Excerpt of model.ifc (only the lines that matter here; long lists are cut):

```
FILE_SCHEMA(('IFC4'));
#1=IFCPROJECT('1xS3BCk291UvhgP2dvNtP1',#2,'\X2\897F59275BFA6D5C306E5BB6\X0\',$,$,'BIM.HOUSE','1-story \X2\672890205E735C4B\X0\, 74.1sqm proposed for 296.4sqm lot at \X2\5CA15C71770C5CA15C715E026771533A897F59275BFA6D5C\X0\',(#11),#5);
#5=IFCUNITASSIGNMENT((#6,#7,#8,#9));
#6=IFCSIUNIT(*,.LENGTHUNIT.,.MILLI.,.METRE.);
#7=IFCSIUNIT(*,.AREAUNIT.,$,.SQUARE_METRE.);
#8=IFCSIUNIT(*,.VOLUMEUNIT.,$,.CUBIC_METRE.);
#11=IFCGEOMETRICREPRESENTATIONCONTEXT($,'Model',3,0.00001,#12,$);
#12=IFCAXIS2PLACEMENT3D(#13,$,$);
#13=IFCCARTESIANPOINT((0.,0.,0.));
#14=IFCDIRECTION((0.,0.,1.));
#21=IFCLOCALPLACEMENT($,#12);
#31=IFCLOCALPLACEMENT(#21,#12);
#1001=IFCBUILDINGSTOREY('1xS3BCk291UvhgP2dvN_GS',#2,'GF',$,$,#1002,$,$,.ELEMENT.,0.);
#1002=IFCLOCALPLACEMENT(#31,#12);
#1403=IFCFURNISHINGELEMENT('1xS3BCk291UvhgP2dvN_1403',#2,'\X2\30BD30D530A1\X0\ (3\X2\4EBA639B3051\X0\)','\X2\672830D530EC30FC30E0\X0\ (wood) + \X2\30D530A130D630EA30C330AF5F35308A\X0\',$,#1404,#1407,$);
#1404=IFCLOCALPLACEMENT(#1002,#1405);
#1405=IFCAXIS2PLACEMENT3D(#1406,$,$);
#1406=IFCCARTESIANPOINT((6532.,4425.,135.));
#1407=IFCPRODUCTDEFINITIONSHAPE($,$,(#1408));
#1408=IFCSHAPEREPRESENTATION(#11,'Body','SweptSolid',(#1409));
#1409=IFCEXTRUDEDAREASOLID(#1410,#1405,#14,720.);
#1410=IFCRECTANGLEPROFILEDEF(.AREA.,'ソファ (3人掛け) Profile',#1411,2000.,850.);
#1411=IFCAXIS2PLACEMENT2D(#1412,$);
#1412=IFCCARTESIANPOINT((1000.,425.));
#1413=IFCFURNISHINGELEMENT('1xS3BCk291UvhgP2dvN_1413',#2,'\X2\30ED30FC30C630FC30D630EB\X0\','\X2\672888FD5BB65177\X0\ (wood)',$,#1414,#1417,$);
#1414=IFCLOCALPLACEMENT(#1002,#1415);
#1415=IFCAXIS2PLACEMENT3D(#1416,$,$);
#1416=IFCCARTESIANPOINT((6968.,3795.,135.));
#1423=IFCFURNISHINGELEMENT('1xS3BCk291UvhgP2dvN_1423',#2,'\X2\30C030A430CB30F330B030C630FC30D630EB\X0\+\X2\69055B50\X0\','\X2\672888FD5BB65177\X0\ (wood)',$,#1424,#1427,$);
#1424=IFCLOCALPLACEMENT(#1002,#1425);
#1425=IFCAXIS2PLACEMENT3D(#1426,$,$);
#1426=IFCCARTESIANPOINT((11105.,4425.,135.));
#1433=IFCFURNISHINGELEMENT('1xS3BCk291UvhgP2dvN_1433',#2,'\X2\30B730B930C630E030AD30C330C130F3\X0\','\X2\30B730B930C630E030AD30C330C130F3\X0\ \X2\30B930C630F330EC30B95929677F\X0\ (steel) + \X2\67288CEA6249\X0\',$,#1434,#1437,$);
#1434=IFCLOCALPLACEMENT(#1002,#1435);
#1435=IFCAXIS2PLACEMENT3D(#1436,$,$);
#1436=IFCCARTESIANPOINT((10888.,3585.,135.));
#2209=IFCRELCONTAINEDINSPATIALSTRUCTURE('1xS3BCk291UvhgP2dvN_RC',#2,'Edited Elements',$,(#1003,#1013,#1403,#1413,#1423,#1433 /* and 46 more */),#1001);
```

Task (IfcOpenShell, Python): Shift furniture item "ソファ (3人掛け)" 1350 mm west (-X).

```python
import ifcopenshell
import ifcopenshell.api.geometry
import ifcopenshell.util.placement
import ifcopenshell.util.unit

model = ifcopenshell.open("model.ifc")
unit_scale = ifcopenshell.util.unit.calculate_unit_scale(model)

item = model.by_guid("1xS3BCk291UvhgP2dvN_1403")
matrix = ifcopenshell.util.placement.get_local_placement(item.ObjectPlacement)
matrix[0, 3] -= 1.35 / unit_scale
ifcopenshell.api.geometry.edit_object_placement(model, product=item, matrix=matrix, is_si=False)

print(ifcopenshell.util.placement.get_local_placement(item.ObjectPlacement).round(3) + 0.0)

model.write("model_v2.ifc")
```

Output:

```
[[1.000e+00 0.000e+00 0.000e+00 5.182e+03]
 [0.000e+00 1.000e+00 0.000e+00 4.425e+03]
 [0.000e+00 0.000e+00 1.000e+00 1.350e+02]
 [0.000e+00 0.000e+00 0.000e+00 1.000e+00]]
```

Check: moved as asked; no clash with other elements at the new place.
